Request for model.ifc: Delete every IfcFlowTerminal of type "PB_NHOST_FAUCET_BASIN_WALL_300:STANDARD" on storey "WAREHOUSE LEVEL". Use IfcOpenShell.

First a look at what the model holds.

```python
import ifcopenshell
import ifcopenshell.util.element

model = ifcopenshell.open("model.ifc")
print(model.schema)
storey = next(s for s in model.by_type("IfcBuildingStorey") if s.Name == "WAREHOUSE LEVEL")
terminals = [e for e in ifcopenshell.util.element.get_decomposition(storey) if e.is_a("IfcFlowTerminal")]
seen = {}
for e in terminals:
    element_type = ifcopenshell.util.element.get_type(e)
    name = element_type.Name if element_type not in (None, e) else None
    seen[name] = seen.get(name, 0) + 1
for name, count in sorted(seen.items(), key=str):
    print(count, "x", name)
```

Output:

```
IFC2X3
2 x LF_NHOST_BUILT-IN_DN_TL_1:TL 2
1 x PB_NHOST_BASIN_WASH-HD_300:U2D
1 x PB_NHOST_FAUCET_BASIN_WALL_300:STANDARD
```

```python
import ifcopenshell
import ifcopenshell.api.root
import ifcopenshell.util.element

model = ifcopenshell.open("model.ifc")

storey = next(s for s in model.by_type("IfcBuildingStorey") if s.Name == "WAREHOUSE LEVEL")
terminals = [e for e in ifcopenshell.util.element.get_decomposition(storey) if e.is_a("IfcFlowTerminal")]
targets = [e for e in terminals if (t := ifcopenshell.util.element.get_type(e)) not in (None, e) and t.Name == "PB_NHOST_FAUCET_BASIN_WALL_300:STANDARD"]

for e in targets:
    ifcopenshell.api.root.remove_product(model, product=e)
print(len(targets), "removed")

model.write("model_updated.ifc")
```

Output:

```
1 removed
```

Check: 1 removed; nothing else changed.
